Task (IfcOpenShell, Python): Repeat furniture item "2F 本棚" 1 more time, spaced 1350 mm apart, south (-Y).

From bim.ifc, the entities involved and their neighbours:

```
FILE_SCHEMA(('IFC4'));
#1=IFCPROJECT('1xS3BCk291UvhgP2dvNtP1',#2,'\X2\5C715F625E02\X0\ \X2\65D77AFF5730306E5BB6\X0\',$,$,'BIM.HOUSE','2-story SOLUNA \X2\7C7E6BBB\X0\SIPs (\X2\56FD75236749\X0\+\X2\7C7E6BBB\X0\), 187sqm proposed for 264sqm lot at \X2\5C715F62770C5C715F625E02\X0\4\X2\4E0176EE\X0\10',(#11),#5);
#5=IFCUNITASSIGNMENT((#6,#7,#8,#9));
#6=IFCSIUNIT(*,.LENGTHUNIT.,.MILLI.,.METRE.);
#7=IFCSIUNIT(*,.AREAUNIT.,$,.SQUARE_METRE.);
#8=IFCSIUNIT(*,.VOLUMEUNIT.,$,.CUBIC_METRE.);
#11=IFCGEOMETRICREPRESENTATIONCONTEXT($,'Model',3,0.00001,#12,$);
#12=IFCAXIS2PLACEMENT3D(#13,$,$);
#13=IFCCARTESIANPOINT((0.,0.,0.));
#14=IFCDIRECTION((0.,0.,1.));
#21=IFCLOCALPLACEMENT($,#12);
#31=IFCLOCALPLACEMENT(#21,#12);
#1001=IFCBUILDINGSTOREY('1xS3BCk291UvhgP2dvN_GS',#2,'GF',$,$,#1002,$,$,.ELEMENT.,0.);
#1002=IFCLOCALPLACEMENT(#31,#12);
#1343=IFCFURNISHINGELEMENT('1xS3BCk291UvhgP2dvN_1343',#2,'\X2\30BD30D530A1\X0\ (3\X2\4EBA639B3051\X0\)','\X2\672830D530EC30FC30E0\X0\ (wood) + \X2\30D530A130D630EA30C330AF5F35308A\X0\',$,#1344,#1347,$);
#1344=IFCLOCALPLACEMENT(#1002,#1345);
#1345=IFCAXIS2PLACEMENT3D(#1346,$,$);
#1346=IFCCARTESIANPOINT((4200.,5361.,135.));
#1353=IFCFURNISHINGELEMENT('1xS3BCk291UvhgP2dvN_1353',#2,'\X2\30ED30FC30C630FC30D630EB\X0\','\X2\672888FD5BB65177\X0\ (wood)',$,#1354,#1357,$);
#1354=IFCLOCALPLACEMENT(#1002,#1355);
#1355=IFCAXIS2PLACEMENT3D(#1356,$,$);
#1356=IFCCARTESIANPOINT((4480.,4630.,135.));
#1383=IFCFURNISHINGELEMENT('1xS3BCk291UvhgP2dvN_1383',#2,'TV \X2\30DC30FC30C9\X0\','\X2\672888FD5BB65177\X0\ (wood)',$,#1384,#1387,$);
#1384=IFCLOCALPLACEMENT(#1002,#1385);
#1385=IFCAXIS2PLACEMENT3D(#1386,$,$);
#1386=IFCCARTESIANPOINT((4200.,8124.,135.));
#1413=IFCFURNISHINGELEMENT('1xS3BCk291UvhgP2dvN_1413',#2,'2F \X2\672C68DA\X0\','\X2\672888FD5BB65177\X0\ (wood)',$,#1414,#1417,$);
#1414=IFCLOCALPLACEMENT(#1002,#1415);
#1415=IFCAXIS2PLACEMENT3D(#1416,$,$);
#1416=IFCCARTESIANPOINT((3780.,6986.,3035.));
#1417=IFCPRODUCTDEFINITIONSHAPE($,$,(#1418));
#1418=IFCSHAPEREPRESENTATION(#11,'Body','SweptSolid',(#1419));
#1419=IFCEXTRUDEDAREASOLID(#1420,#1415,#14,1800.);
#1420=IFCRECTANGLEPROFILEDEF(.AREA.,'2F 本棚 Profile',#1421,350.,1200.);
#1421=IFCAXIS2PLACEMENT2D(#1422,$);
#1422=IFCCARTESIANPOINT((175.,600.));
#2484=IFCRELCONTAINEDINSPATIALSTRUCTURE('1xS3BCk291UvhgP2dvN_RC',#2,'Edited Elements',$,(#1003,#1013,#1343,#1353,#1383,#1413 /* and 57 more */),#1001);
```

```python
import numpy as np
import ifcopenshell
import ifcopenshell.api.geometry
import ifcopenshell.api.root
import ifcopenshell.util.element
import ifcopenshell.util.placement
import ifcopenshell.util.unit

model = ifcopenshell.open("bim.ifc")
unit_scale = ifcopenshell.util.unit.calculate_unit_scale(model)


def reuse_history(source, copy):
    """copy_class also copies each property set's owner history, people and application; keep the originals."""
    for rel in copy.IsDefinedBy:
        if rel.is_a("IfcRelDefinesByProperties") and (history := rel.RelatingPropertyDefinition.OwnerHistory):
            rel.RelatingPropertyDefinition.OwnerHistory = source.OwnerHistory
            ifcopenshell.util.element.remove_deep2(model, history)


source = model.by_id(1413)
base = ifcopenshell.util.placement.get_local_placement(source.ObjectPlacement)
step = np.array([0.0, -1.0, 0.0]) * 1.35 / unit_scale

for i in range(1, 2):
    copy = ifcopenshell.api.root.copy_class(model, product=source)
    copy.Representation = ifcopenshell.util.element.copy_deep(
        model, source.Representation, exclude=["IfcGeometricRepresentationContext", "IfcRepresentationMap"]
    )
    reuse_history(source, copy)
    matrix = base.copy()
    matrix[:3, 3] += i * step
    print("added at", matrix[:3, 3].round(3) + 0.0)
    ifcopenshell.api.geometry.edit_object_placement(model, product=copy, matrix=matrix, is_si=False)

model.write("bim_rev.ifc")
```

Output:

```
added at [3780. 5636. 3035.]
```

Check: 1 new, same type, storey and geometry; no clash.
